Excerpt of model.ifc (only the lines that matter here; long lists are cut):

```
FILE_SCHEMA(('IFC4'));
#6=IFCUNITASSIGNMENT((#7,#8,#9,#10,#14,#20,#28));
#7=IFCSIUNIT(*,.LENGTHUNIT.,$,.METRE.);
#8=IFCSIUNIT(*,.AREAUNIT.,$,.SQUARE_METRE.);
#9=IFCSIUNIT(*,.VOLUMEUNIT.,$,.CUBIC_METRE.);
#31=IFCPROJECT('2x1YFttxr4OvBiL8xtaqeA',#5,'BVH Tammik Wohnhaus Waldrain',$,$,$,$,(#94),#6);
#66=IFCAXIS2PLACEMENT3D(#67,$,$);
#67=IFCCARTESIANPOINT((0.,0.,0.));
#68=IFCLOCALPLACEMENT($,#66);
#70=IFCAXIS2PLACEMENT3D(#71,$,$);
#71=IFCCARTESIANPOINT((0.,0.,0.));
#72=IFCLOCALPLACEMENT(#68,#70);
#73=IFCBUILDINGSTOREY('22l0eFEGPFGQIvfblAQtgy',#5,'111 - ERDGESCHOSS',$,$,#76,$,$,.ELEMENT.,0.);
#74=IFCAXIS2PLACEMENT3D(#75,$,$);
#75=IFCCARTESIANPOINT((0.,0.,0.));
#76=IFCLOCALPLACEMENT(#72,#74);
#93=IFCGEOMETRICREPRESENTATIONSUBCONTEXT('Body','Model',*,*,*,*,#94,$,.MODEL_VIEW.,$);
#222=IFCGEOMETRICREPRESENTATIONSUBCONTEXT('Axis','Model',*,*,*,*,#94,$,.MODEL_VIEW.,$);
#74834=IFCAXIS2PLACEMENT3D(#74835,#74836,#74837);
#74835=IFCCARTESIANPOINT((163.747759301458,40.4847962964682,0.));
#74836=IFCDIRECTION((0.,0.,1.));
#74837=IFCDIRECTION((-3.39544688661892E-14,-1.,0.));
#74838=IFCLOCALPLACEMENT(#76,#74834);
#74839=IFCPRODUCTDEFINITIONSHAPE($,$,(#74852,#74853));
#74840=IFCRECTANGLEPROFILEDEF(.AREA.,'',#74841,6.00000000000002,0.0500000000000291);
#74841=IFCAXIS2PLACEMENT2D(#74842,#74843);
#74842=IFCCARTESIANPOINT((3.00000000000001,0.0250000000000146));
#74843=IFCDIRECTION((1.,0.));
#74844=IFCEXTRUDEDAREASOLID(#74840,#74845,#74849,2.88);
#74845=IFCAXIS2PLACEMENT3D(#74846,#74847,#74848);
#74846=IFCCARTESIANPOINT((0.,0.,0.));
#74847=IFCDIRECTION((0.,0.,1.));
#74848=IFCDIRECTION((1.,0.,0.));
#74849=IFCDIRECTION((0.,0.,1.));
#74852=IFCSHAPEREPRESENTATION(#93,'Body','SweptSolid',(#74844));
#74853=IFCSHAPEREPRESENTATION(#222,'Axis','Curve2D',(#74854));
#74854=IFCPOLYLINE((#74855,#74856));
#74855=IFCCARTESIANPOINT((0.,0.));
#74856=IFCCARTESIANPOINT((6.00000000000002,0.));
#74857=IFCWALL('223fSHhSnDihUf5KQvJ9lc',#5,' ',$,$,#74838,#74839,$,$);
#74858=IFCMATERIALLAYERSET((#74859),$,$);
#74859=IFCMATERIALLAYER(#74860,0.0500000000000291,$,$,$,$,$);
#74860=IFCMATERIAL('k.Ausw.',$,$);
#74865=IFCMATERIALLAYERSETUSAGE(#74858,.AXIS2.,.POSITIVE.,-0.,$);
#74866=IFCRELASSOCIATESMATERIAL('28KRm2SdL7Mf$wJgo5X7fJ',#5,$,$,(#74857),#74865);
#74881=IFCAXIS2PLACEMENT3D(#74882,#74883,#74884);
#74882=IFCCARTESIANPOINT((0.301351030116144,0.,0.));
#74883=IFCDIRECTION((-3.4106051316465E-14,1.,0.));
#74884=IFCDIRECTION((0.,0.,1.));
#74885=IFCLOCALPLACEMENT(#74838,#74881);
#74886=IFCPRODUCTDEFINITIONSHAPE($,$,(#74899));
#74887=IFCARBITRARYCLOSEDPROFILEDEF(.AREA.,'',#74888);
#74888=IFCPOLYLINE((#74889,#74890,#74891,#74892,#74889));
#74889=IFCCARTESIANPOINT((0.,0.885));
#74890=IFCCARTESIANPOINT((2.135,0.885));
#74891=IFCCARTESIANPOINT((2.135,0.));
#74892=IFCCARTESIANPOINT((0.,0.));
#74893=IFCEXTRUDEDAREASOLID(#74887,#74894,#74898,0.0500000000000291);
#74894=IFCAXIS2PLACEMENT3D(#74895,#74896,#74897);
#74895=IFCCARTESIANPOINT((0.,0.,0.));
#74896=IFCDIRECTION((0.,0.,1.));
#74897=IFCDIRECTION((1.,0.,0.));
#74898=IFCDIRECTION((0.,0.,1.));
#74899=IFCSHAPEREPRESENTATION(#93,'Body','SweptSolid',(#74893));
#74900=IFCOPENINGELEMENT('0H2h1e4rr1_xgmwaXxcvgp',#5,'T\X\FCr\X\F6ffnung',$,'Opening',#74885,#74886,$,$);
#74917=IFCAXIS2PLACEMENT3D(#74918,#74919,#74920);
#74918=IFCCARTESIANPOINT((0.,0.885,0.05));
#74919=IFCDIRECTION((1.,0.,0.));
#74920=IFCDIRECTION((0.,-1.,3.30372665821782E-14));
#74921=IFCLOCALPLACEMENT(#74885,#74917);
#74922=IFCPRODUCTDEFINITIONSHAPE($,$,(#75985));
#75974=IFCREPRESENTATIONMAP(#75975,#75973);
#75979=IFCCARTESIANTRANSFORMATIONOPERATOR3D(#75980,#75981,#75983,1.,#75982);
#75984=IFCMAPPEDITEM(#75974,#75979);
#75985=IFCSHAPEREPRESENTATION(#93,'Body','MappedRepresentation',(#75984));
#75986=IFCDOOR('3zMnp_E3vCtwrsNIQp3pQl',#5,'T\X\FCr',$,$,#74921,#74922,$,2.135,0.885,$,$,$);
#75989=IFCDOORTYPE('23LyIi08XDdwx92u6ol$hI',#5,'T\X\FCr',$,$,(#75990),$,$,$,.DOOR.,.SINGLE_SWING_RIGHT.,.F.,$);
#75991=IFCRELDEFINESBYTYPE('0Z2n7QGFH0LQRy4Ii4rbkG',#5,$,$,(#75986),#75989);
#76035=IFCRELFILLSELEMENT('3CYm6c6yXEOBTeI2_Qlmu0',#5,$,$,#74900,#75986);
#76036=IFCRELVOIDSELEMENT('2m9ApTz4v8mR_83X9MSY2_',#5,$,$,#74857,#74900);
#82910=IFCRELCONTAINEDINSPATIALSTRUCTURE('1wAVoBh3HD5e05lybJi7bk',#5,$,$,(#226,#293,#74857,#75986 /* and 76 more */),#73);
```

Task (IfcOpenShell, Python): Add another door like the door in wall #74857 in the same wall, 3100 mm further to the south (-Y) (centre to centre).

```python
import ifcopenshell
import ifcopenshell.api.feature
import ifcopenshell.api.geometry
import ifcopenshell.api.root
import ifcopenshell.geom
import ifcopenshell.util.element
import ifcopenshell.util.placement
import ifcopenshell.util.shape

model = ifcopenshell.open("model.ifc")
settings = ifcopenshell.geom.settings()


def volume(element):
    """Net volume in cubic metres, openings subtracted."""
    shape = ifcopenshell.geom.create_shape(settings, element)
    return ifcopenshell.util.shape.get_volume(shape.geometry)


def reuse_history(source, copy):
    """copy_class also copies each property set's owner history, people and application; keep the originals."""
    for rel in copy.IsDefinedBy:
        if rel.is_a("IfcRelDefinesByProperties") and (history := rel.RelatingPropertyDefinition.OwnerHistory):
            rel.RelatingPropertyDefinition.OwnerHistory = source.OwnerHistory
            ifcopenshell.util.element.remove_deep2(model, history)


door = model.by_guid("3zMnp_E3vCtwrsNIQp3pQl")
opening = door.FillsVoids[0].RelatingOpeningElement
wall = opening.VoidsElements[0].RelatingBuildingElement
before = volume(wall)
shift = ifcopenshell.util.placement.get_local_placement(wall.ObjectPlacement)[:3, 0] * 3.1

# copy_class copies the void relationship, type, container and properties, but no geometry.
new_opening = ifcopenshell.api.root.copy_class(model, product=opening)
new_opening.Representation = ifcopenshell.util.element.copy_deep(
    model, opening.Representation, exclude=["IfcGeometricRepresentationContext", "IfcRepresentationMap"]
)
reuse_history(opening, new_opening)
new_door = ifcopenshell.api.root.copy_class(model, product=door)
new_door.Representation = ifcopenshell.util.element.copy_deep(
    model, door.Representation, exclude=["IfcGeometricRepresentationContext", "IfcRepresentationMap"]
)
reuse_history(door, new_door)
ifcopenshell.api.feature.add_filling(model, opening=new_opening, element=new_door)

for old, new in ((opening, new_opening), (door, new_door)):
    matrix = ifcopenshell.util.placement.get_local_placement(old.ObjectPlacement)
    matrix[:3, 3] += shift
    ifcopenshell.api.geometry.edit_object_placement(model, product=new, matrix=matrix, is_si=False)

after = volume(wall)

print(f"wall volume {before:.3f} -> {after:.3f} m3")

model.write("model_updated.ifc")
```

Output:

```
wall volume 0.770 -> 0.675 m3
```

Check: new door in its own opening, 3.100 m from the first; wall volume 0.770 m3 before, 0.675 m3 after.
